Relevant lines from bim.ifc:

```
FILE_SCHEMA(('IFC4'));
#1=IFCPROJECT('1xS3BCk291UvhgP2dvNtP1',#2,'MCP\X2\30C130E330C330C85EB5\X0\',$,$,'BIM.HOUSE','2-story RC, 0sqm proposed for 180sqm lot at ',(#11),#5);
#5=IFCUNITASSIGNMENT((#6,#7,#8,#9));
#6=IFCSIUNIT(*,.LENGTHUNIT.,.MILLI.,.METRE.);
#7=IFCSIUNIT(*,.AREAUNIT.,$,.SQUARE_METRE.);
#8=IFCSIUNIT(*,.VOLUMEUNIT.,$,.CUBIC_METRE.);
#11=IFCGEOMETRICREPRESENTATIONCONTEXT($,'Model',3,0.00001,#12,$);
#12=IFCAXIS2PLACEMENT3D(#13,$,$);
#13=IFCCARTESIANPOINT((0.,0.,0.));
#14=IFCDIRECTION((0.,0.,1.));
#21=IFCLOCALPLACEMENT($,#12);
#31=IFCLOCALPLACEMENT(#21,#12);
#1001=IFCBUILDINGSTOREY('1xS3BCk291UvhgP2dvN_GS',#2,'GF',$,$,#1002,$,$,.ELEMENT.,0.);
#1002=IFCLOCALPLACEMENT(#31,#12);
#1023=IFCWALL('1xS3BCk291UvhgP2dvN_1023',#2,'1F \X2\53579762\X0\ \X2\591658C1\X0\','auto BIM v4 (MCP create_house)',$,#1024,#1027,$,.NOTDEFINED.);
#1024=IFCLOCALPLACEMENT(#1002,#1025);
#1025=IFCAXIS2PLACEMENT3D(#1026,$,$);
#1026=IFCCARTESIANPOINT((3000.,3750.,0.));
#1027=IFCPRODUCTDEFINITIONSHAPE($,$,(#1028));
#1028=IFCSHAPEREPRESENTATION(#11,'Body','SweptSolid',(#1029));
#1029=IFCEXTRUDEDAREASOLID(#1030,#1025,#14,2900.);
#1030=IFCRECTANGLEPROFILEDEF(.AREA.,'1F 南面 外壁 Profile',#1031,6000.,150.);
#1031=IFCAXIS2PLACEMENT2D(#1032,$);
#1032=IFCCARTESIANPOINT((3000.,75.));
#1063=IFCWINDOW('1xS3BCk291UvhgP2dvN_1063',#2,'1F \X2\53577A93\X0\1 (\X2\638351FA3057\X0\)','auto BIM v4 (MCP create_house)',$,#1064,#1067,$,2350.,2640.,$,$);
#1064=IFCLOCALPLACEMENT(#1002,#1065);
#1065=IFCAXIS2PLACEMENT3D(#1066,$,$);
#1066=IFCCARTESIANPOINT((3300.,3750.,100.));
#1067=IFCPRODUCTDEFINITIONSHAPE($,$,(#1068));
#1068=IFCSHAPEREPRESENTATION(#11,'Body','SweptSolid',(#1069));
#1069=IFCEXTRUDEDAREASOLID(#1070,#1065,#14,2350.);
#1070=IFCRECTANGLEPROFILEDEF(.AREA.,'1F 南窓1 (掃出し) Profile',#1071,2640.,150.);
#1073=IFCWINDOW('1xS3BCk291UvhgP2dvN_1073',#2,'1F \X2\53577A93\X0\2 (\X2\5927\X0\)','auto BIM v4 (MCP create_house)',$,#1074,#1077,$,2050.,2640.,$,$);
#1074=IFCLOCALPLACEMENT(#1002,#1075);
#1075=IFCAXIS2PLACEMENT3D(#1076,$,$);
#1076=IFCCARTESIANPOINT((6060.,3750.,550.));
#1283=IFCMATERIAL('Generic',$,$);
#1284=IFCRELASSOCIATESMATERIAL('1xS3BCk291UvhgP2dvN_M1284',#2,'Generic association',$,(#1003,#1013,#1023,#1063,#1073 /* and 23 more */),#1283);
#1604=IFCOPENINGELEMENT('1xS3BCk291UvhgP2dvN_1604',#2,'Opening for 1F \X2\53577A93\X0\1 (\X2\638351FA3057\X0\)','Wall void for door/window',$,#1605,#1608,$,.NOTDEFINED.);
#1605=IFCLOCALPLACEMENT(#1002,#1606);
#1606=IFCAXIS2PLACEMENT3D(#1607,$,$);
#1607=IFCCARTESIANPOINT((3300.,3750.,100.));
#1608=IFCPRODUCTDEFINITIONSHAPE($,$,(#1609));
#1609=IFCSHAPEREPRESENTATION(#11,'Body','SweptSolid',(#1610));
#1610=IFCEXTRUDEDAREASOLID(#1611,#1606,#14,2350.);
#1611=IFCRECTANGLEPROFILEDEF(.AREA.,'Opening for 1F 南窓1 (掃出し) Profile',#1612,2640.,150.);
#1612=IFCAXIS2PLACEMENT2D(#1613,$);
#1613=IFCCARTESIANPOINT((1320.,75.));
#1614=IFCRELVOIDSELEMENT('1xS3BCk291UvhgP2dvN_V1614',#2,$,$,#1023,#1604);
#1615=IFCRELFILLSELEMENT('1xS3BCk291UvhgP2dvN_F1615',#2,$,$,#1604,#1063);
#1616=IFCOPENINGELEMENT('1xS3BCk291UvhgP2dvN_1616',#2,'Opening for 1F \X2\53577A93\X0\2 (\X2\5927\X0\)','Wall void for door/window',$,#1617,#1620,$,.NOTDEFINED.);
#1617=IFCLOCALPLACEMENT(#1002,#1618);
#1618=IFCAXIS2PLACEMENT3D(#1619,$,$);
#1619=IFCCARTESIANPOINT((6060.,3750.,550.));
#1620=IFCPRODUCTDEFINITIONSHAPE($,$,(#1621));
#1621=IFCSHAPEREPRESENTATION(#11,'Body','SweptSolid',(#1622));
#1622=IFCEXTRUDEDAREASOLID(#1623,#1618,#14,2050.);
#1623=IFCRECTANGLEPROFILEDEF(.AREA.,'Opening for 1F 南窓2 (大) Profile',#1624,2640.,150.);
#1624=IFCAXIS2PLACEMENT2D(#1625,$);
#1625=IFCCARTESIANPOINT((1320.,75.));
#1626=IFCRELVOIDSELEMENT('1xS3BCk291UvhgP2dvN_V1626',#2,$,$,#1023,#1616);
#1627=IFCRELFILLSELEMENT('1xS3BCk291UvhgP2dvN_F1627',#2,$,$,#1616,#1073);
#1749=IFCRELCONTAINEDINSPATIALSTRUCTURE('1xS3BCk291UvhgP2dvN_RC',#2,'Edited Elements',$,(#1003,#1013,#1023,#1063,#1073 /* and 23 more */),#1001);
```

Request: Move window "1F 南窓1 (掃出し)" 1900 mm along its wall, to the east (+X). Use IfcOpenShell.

```python
import ifcopenshell
import ifcopenshell.api.geometry
import ifcopenshell.util.placement

model = ifcopenshell.open("bim.ifc")

window = model.by_id(1063)
opening = window.FillsVoids[0].RelatingOpeningElement
wall = opening.VoidsElements[0].RelatingBuildingElement

wall_matrix = ifcopenshell.util.placement.get_local_placement(wall.ObjectPlacement)
shift = wall_matrix[:3, 0] * 1900.0
before = ifcopenshell.util.placement.get_local_placement(window.ObjectPlacement)[:3, 3].copy()

# The window is not placed relative to its opening, so move both.
for product in (opening, window):
    matrix = ifcopenshell.util.placement.get_local_placement(product.ObjectPlacement)
    matrix[:3, 3] += shift
    ifcopenshell.api.geometry.edit_object_placement(model, product=product, matrix=matrix, is_si=False)

after = ifcopenshell.util.placement.get_local_placement(window.ObjectPlacement)[:3, 3]
print("window moved by", (after - before).round(3) + 0.0)

model.write("bim_edited.ifc")
```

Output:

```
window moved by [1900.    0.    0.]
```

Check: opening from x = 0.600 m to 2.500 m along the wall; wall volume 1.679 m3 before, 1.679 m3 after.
